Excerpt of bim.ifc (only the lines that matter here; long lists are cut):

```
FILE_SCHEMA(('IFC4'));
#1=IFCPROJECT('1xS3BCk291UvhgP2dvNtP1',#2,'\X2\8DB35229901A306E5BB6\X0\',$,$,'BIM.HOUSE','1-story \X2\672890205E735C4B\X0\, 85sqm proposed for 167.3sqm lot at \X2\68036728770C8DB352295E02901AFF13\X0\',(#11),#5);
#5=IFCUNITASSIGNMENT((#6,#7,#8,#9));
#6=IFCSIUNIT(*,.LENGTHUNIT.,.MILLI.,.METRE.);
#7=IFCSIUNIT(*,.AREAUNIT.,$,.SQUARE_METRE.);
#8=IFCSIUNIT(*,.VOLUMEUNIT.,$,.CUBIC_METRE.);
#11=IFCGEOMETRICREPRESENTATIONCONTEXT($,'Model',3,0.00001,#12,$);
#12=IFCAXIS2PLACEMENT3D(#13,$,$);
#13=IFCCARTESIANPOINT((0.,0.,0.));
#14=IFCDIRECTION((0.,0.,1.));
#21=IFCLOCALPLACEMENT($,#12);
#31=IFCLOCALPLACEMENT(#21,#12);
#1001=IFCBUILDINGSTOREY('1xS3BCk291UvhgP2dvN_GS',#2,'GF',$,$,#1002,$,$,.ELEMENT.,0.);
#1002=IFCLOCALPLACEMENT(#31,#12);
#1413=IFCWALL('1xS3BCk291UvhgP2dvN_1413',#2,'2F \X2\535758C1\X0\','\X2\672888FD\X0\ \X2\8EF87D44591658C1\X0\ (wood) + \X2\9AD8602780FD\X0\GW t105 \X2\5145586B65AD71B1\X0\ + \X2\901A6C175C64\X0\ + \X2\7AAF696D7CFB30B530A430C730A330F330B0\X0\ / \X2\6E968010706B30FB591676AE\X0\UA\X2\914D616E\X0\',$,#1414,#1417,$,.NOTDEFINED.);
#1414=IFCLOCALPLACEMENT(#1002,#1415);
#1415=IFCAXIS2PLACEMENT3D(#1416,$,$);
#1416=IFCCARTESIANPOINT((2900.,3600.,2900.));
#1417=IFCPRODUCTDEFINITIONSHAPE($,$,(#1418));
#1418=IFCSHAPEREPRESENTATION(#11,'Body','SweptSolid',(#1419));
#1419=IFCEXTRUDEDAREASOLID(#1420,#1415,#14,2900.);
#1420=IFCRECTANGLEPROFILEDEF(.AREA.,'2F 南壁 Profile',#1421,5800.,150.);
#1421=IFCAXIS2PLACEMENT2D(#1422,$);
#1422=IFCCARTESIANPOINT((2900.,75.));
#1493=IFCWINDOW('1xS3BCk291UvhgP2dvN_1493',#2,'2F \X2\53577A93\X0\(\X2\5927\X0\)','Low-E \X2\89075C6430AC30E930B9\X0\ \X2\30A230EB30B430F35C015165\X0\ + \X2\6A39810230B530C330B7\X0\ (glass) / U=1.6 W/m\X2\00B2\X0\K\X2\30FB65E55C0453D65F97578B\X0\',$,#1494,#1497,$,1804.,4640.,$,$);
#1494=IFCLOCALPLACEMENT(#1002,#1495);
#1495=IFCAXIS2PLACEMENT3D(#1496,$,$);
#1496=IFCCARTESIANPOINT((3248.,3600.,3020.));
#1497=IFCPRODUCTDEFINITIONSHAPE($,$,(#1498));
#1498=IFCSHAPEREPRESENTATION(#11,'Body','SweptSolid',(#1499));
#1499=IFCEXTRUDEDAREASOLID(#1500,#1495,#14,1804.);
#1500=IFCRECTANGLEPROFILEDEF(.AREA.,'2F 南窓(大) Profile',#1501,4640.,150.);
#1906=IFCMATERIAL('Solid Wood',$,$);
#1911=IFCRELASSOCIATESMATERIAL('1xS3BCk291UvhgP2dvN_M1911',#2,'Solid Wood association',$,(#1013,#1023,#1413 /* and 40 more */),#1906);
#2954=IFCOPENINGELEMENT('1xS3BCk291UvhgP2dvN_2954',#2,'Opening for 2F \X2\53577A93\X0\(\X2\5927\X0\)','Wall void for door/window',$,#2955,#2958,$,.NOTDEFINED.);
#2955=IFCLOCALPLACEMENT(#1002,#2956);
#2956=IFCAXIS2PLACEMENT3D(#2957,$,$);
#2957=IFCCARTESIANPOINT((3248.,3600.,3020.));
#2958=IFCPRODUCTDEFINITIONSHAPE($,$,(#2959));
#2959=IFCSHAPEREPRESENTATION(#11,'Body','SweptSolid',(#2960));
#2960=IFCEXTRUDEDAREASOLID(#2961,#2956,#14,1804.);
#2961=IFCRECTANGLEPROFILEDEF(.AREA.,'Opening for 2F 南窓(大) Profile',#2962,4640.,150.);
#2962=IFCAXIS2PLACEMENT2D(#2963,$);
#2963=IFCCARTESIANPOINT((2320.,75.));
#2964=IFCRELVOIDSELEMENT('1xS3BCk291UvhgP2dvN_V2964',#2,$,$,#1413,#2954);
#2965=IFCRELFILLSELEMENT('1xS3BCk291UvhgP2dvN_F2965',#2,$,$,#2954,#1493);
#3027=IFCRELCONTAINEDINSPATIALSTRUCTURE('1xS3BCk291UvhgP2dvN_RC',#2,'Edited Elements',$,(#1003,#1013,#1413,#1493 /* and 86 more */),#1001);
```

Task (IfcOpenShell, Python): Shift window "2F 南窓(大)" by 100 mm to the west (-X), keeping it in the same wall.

```python
import ifcopenshell
import ifcopenshell.api.geometry
import ifcopenshell.util.placement

model = ifcopenshell.open("bim.ifc")

window = model.by_guid("1xS3BCk291UvhgP2dvN_1493")
opening = window.FillsVoids[0].RelatingOpeningElement
wall = opening.VoidsElements[0].RelatingBuildingElement

wall_matrix = ifcopenshell.util.placement.get_local_placement(wall.ObjectPlacement)
shift = wall_matrix[:3, 0] * -100.0
before = ifcopenshell.util.placement.get_local_placement(window.ObjectPlacement)[:3, 3].copy()

# The window is not placed relative to its opening, so move both.
for product in (opening, window):
    matrix = ifcopenshell.util.placement.get_local_placement(product.ObjectPlacement)
    matrix[:3, 3] += shift
    ifcopenshell.api.geometry.edit_object_placement(model, product=product, matrix=matrix, is_si=False)

after = ifcopenshell.util.placement.get_local_placement(window.ObjectPlacement)[:3, 3]
print("window moved by", (after - before).round(3) + 0.0)

model.write("bim_rev.ifc")
```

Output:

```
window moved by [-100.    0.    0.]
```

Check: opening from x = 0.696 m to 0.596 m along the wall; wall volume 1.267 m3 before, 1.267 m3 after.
